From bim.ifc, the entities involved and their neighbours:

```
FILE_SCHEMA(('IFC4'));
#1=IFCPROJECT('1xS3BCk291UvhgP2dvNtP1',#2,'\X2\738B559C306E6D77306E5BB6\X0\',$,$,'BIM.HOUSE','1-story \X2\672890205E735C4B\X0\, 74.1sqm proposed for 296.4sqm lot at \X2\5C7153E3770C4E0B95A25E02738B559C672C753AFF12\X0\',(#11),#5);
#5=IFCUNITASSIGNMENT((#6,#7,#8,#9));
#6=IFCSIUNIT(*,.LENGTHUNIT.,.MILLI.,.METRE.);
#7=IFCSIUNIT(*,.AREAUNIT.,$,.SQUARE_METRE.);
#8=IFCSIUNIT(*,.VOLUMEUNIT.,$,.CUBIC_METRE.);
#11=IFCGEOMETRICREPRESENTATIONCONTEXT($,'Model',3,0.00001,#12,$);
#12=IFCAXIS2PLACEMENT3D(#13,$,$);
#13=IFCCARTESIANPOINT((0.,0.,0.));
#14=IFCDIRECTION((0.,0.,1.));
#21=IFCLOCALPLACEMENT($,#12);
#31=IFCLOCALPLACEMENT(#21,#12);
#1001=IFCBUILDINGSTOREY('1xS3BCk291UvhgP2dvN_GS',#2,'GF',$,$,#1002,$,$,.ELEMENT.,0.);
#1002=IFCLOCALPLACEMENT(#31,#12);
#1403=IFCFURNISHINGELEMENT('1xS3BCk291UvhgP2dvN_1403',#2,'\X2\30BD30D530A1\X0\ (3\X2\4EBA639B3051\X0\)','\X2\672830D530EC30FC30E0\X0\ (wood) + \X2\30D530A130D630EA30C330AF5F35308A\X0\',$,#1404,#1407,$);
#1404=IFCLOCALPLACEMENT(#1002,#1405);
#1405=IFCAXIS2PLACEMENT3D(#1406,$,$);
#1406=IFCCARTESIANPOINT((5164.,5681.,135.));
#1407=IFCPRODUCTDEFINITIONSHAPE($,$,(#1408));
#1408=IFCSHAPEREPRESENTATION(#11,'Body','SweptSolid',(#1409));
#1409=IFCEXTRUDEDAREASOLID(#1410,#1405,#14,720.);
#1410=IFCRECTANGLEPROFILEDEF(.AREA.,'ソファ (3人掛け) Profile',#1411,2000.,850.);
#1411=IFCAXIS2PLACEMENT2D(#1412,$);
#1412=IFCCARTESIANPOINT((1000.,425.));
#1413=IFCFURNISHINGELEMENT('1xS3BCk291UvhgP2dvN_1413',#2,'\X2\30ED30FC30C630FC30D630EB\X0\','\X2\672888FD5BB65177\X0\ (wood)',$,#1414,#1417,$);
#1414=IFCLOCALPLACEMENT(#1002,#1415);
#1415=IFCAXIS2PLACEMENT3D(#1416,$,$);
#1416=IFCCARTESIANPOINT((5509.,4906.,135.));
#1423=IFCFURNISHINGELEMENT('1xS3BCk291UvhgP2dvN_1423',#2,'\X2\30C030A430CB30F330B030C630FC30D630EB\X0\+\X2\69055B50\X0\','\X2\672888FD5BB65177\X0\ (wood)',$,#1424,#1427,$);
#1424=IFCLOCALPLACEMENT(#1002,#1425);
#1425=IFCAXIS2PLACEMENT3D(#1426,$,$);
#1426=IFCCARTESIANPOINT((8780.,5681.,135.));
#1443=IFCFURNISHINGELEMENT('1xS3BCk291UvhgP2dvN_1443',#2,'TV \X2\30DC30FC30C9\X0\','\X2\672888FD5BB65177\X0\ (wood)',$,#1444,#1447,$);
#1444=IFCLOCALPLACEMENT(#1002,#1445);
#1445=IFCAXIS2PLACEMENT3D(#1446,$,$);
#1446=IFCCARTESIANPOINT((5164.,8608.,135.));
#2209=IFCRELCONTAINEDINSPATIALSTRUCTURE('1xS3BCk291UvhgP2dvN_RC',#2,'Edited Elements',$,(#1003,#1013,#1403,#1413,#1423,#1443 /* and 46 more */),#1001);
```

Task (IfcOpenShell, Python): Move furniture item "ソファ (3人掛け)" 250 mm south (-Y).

```python
import ifcopenshell
import ifcopenshell.api.geometry
import ifcopenshell.util.placement
import ifcopenshell.util.unit

model = ifcopenshell.open("bim.ifc")
unit_scale = ifcopenshell.util.unit.calculate_unit_scale(model)

item = model.by_id(1403)
matrix = ifcopenshell.util.placement.get_local_placement(item.ObjectPlacement)
matrix[1, 3] -= 0.25 / unit_scale
ifcopenshell.api.geometry.edit_object_placement(model, product=item, matrix=matrix, is_si=False)

print(ifcopenshell.util.placement.get_local_placement(item.ObjectPlacement).round(3) + 0.0)

model.write("bim_v2.ifc")
```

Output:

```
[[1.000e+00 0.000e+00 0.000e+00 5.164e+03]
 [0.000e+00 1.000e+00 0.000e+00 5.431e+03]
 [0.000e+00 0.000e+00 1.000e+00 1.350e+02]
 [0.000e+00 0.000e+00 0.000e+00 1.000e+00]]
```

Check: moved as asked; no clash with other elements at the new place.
